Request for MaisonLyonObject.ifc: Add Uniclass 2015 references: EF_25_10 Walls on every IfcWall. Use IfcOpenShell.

First a look at what the model holds.

```python
import ifcopenshell

model = ifcopenshell.open("MaisonLyonObject.ifc")
print(model.schema)
print("classifications:", [c.Name for c in model.by_type("IfcClassification")])
for ifc_class in ("IfcDoor", "IfcRoof", "IfcStair", "IfcWall", "IfcWindow"):
    print(ifc_class, len(model.by_type(ifc_class)))
```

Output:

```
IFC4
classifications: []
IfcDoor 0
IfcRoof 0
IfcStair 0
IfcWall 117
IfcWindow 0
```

```python
import ifcopenshell
import ifcopenshell.api.classification

model = ifcopenshell.open("MaisonLyonObject.ifc")

system = ifcopenshell.api.classification.add_classification(model, classification="Uniclass 2015")

codes = {
    "IfcWall": ("EF_25_10", "Walls"),
}
for ifc_class, (code, name) in codes.items():
    products = model.by_type(ifc_class)
    ifcopenshell.api.classification.add_reference(
        model, products=products, classification=system, identification=code, name=name
    )
    print(code, len(products))

model.write("MaisonLyonObject_updated.ifc")
```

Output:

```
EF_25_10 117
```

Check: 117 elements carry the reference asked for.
